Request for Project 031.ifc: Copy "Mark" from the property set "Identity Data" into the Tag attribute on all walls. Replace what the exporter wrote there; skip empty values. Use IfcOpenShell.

First a look at what the model holds.

```python
import ifcopenshell
import ifcopenshell.util.element

model = ifcopenshell.open("Project 031.ifc")
print(model.schema)
walls = model.by_type("IfcWall")
print(len(walls), "walls")
for e in walls[:8]:
    source = ifcopenshell.util.element.get_pset(e, "Identity Data", "Mark")
    target = e.Tag
    print(e.id(), repr(source), repr(target), sep=" | ")
```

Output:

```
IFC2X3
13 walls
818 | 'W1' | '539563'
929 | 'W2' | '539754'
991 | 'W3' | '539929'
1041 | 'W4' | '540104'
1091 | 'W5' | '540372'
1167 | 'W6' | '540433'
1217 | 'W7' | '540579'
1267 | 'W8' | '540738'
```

```python
import ifcopenshell
import ifcopenshell.util.element

model = ifcopenshell.open("Project 031.ifc")

count = 0
for e in model.by_type("IfcWall"):
    value = ifcopenshell.util.element.get_pset(e, "Identity Data", "Mark")
    current = e.Tag
    if not value or not value.strip() or current == value:
        continue
    e.Tag = value
    count += 1

print(count, "walls updated")

model.write("Project 031-out.ifc")
```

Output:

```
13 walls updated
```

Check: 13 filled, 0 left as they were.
